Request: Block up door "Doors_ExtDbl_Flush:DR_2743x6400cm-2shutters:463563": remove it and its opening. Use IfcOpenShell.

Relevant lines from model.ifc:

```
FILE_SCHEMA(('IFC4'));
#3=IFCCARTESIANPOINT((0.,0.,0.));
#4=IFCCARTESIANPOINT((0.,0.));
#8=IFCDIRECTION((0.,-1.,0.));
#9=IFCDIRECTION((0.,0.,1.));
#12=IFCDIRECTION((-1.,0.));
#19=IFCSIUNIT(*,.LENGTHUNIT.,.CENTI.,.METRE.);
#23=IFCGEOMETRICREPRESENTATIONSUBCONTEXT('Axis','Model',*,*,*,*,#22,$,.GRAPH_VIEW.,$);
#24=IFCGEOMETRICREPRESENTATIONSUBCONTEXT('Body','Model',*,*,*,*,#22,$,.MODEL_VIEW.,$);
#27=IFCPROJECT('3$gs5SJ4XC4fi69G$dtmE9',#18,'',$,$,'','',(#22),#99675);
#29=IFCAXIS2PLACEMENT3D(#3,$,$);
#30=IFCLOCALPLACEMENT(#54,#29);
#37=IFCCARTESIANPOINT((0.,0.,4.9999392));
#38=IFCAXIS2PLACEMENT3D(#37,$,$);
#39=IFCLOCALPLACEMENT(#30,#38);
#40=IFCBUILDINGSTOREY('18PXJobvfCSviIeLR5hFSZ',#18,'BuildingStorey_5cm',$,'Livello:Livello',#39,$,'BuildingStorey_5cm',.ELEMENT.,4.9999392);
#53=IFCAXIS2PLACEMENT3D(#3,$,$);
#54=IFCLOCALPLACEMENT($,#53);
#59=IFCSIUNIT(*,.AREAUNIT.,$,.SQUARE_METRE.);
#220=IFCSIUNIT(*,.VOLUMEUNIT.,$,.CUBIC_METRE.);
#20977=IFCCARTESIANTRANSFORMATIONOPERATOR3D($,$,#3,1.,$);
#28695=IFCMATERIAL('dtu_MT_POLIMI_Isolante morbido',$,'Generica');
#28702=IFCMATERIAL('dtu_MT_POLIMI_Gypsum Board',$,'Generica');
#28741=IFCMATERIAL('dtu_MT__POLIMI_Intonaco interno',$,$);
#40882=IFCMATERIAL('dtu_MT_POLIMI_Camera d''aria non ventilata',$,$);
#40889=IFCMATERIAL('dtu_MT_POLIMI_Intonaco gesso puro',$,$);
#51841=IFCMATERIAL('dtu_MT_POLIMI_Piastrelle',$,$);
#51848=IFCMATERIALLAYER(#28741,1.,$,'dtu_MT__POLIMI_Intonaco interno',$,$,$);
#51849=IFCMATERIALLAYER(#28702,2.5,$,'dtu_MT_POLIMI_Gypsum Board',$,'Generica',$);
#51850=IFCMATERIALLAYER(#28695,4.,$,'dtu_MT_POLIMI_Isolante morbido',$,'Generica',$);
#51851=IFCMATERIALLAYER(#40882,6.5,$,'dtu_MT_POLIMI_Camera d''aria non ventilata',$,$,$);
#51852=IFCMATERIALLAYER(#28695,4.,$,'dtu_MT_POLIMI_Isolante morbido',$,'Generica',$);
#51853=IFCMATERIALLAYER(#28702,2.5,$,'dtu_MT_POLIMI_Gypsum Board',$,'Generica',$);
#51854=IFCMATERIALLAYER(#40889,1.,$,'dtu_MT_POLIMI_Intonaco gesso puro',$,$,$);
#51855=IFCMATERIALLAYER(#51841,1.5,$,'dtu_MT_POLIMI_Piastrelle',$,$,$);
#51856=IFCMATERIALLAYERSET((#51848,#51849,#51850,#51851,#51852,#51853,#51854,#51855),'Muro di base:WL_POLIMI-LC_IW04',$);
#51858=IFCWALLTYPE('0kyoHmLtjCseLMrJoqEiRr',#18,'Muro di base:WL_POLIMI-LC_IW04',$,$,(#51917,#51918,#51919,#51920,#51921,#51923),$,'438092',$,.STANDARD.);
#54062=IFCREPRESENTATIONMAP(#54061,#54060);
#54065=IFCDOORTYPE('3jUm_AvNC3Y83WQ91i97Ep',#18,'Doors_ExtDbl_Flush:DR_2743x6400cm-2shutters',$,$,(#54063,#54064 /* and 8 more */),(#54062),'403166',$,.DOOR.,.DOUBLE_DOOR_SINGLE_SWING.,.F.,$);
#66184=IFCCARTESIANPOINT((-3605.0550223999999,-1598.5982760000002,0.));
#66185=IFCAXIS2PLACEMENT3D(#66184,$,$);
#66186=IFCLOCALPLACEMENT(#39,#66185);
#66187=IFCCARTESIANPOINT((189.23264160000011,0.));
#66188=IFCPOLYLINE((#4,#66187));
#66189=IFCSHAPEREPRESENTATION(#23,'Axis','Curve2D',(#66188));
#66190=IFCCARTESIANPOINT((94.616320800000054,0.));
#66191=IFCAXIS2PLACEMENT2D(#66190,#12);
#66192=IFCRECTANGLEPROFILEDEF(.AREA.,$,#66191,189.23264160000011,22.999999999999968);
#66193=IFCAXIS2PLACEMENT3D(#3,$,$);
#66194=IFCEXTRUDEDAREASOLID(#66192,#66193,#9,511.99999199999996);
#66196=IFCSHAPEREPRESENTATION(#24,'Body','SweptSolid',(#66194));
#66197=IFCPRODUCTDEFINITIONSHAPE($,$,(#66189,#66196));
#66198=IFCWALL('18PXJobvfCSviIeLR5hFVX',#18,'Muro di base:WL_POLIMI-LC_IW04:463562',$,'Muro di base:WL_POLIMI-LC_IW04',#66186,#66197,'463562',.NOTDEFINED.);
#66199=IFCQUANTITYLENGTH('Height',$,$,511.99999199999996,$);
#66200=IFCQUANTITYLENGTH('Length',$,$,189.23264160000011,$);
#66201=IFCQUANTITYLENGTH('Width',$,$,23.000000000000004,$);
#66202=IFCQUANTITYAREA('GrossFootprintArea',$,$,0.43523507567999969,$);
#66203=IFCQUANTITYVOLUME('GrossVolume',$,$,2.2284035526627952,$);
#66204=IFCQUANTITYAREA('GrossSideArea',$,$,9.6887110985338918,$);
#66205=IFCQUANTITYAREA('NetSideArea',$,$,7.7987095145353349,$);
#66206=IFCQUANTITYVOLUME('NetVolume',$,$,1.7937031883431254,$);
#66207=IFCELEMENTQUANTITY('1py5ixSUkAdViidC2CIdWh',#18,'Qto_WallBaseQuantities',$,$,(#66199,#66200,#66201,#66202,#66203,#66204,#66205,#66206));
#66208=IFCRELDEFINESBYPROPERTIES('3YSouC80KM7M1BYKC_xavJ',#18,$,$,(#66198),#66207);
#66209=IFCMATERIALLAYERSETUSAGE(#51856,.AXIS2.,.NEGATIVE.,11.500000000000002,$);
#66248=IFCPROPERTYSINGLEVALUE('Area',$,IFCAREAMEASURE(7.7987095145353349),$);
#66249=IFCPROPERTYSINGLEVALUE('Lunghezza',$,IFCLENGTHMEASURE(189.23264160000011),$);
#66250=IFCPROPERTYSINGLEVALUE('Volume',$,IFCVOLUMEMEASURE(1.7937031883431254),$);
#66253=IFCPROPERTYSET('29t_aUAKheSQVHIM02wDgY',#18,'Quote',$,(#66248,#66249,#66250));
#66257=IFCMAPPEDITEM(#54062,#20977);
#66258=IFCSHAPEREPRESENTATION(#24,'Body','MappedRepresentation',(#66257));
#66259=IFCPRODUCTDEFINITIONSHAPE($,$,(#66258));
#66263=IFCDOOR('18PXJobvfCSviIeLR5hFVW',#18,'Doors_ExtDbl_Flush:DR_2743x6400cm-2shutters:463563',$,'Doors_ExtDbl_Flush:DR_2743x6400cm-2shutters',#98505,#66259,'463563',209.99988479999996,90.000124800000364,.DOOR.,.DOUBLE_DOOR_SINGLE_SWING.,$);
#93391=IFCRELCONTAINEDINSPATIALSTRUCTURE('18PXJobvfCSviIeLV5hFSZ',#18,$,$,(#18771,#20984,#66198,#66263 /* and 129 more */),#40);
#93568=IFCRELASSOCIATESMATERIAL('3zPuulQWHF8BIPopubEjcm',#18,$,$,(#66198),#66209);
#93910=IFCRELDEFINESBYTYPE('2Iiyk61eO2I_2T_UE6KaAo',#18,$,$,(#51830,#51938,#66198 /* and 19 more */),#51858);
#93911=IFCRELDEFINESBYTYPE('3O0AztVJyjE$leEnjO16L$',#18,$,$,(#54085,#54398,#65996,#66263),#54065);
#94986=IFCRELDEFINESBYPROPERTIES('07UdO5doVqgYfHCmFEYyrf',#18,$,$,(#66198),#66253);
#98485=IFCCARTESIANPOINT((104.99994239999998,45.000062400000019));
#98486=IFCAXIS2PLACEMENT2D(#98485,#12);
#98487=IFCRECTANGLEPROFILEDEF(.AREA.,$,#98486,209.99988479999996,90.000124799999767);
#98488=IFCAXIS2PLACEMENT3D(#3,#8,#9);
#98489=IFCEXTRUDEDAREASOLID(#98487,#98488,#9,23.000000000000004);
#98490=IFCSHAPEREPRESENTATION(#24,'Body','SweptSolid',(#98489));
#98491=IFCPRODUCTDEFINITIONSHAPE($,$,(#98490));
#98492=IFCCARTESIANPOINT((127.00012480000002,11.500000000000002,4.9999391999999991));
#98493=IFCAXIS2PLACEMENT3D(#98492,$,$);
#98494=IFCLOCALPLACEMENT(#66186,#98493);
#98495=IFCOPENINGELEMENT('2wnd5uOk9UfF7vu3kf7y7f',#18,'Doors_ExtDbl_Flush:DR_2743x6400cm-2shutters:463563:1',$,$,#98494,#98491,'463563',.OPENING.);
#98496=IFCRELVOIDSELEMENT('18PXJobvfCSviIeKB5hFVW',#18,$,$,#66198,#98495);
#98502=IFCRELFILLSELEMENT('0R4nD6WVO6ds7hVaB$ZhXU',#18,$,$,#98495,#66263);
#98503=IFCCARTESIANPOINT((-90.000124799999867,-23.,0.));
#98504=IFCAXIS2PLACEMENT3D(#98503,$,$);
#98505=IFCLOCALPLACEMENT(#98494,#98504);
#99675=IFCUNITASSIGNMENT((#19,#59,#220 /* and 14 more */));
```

```python
import ifcopenshell
import ifcopenshell.api.feature
import ifcopenshell.api.pset
import ifcopenshell.api.root
import ifcopenshell.geom
import ifcopenshell.util.element
import ifcopenshell.util.shape
import ifcopenshell.util.unit

model = ifcopenshell.open("model.ifc")
area_scale = ifcopenshell.util.unit.calculate_unit_scale(model, "AREAUNIT")
volume_scale = ifcopenshell.util.unit.calculate_unit_scale(model, "VOLUMEUNIT")
settings = ifcopenshell.geom.settings()


def volume(element):
    """Net volume in cubic metres, openings subtracted."""
    shape = ifcopenshell.geom.create_shape(settings, element)
    return ifcopenshell.util.shape.get_volume(shape.geometry)


door = model.by_guid("18PXJobvfCSviIeLR5hFVW")
opening = door.FillsVoids[0].RelatingOpeningElement
wall = opening.VoidsElements[0].RelatingBuildingElement
before = volume(wall)

ifcopenshell.api.root.remove_product(model, product=door)
ifcopenshell.api.feature.remove_feature(model, feature=opening)

after = volume(wall)
thickness = 0.23  # wall thickness in metres

# Update the wall's stored quantities.
qto = model.by_id(ifcopenshell.util.element.get_pset(wall, "Qto_WallBaseQuantities", should_inherit=False)["id"])
ifcopenshell.api.pset.edit_qto(model, qto=qto, properties={
    "NetSideArea": after / thickness / area_scale,
    "NetVolume": after / volume_scale,
})
pset = model.by_id(ifcopenshell.util.element.get_pset(wall, "Quote", should_inherit=False)["id"])
ifcopenshell.api.pset.edit_pset(model, pset=pset, properties={
    "Area": model.create_entity("IfcAreaMeasure", after / thickness / area_scale),
    "Volume": model.create_entity("IfcVolumeMeasure", after / volume_scale),
})

print(f"wall volume {before:.3f} -> {after:.3f} m3")

model.write("model_updated.ifc")
```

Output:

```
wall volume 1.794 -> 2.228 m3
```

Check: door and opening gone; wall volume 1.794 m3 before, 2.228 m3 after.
